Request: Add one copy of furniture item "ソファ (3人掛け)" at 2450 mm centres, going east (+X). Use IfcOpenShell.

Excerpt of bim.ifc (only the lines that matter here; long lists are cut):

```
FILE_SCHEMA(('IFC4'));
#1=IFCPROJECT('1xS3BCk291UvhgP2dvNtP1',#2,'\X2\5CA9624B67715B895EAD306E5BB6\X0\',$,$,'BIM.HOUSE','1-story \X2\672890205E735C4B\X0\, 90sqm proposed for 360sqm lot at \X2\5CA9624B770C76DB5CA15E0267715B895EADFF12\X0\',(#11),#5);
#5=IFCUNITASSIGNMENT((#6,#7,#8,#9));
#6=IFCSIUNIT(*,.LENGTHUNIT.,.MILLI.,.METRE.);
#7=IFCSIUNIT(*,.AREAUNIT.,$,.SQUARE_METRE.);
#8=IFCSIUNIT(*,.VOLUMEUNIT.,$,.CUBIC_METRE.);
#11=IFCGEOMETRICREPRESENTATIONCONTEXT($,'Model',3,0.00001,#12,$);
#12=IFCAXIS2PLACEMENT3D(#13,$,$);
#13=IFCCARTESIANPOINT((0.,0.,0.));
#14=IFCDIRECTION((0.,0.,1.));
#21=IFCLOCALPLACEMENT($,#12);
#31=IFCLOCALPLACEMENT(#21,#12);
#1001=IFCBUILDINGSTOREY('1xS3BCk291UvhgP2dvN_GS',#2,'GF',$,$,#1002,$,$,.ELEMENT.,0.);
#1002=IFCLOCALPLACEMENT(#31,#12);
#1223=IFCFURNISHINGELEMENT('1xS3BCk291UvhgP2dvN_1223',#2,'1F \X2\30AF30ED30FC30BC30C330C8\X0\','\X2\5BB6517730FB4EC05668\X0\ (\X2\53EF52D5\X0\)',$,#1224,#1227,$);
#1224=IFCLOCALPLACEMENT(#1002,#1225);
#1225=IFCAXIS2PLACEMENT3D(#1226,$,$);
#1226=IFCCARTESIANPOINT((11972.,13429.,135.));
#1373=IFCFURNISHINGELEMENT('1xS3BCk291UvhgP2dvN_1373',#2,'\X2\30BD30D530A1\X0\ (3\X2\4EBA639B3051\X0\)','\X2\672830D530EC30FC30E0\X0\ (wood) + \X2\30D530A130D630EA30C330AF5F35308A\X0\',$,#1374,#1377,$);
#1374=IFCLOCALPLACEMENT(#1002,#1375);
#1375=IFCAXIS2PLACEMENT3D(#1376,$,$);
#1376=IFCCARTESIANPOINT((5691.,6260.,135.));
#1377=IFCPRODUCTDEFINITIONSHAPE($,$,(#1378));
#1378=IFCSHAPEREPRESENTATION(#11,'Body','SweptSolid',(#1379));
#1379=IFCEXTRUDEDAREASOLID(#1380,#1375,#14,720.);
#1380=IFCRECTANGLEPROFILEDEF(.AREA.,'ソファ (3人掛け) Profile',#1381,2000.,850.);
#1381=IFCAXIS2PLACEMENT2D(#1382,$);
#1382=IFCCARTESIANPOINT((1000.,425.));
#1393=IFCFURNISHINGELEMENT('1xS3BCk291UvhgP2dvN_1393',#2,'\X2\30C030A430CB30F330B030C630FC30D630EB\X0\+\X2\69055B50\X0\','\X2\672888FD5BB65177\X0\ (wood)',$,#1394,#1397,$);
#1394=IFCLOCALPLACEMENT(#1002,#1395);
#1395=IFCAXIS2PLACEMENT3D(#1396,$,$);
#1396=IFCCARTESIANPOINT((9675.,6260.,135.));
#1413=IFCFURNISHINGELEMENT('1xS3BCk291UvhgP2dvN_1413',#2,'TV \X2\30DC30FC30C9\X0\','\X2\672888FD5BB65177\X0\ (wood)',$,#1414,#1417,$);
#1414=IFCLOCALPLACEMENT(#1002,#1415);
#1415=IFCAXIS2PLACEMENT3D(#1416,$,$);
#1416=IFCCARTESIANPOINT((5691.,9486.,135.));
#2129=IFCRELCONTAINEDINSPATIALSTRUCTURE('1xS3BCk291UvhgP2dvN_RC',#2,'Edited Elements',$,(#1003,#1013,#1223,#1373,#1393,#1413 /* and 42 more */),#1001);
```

```python
import numpy as np
import ifcopenshell
import ifcopenshell.api.geometry
import ifcopenshell.api.root
import ifcopenshell.util.element
import ifcopenshell.util.placement
import ifcopenshell.util.unit

model = ifcopenshell.open("bim.ifc")
unit_scale = ifcopenshell.util.unit.calculate_unit_scale(model)


def reuse_history(source, copy):
    """copy_class also copies each property set's owner history, people and application; keep the originals."""
    for rel in copy.IsDefinedBy:
        if rel.is_a("IfcRelDefinesByProperties") and (history := rel.RelatingPropertyDefinition.OwnerHistory):
            rel.RelatingPropertyDefinition.OwnerHistory = source.OwnerHistory
            ifcopenshell.util.element.remove_deep2(model, history)


source = model.by_id(1373)
base = ifcopenshell.util.placement.get_local_placement(source.ObjectPlacement)
step = np.array([1.0, 0.0, 0.0]) * 2.45 / unit_scale

for i in range(1, 2):
    copy = ifcopenshell.api.root.copy_class(model, product=source)
    copy.Representation = ifcopenshell.util.element.copy_deep(
        model, source.Representation, exclude=["IfcGeometricRepresentationContext", "IfcRepresentationMap"]
    )
    reuse_history(source, copy)
    matrix = base.copy()
    matrix[:3, 3] += i * step
    print("added at", matrix[:3, 3].round(3) + 0.0)
    ifcopenshell.api.geometry.edit_object_placement(model, product=copy, matrix=matrix, is_si=False)

model.write("bim_rev.ifc")
```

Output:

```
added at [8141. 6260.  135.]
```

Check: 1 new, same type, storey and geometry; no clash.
